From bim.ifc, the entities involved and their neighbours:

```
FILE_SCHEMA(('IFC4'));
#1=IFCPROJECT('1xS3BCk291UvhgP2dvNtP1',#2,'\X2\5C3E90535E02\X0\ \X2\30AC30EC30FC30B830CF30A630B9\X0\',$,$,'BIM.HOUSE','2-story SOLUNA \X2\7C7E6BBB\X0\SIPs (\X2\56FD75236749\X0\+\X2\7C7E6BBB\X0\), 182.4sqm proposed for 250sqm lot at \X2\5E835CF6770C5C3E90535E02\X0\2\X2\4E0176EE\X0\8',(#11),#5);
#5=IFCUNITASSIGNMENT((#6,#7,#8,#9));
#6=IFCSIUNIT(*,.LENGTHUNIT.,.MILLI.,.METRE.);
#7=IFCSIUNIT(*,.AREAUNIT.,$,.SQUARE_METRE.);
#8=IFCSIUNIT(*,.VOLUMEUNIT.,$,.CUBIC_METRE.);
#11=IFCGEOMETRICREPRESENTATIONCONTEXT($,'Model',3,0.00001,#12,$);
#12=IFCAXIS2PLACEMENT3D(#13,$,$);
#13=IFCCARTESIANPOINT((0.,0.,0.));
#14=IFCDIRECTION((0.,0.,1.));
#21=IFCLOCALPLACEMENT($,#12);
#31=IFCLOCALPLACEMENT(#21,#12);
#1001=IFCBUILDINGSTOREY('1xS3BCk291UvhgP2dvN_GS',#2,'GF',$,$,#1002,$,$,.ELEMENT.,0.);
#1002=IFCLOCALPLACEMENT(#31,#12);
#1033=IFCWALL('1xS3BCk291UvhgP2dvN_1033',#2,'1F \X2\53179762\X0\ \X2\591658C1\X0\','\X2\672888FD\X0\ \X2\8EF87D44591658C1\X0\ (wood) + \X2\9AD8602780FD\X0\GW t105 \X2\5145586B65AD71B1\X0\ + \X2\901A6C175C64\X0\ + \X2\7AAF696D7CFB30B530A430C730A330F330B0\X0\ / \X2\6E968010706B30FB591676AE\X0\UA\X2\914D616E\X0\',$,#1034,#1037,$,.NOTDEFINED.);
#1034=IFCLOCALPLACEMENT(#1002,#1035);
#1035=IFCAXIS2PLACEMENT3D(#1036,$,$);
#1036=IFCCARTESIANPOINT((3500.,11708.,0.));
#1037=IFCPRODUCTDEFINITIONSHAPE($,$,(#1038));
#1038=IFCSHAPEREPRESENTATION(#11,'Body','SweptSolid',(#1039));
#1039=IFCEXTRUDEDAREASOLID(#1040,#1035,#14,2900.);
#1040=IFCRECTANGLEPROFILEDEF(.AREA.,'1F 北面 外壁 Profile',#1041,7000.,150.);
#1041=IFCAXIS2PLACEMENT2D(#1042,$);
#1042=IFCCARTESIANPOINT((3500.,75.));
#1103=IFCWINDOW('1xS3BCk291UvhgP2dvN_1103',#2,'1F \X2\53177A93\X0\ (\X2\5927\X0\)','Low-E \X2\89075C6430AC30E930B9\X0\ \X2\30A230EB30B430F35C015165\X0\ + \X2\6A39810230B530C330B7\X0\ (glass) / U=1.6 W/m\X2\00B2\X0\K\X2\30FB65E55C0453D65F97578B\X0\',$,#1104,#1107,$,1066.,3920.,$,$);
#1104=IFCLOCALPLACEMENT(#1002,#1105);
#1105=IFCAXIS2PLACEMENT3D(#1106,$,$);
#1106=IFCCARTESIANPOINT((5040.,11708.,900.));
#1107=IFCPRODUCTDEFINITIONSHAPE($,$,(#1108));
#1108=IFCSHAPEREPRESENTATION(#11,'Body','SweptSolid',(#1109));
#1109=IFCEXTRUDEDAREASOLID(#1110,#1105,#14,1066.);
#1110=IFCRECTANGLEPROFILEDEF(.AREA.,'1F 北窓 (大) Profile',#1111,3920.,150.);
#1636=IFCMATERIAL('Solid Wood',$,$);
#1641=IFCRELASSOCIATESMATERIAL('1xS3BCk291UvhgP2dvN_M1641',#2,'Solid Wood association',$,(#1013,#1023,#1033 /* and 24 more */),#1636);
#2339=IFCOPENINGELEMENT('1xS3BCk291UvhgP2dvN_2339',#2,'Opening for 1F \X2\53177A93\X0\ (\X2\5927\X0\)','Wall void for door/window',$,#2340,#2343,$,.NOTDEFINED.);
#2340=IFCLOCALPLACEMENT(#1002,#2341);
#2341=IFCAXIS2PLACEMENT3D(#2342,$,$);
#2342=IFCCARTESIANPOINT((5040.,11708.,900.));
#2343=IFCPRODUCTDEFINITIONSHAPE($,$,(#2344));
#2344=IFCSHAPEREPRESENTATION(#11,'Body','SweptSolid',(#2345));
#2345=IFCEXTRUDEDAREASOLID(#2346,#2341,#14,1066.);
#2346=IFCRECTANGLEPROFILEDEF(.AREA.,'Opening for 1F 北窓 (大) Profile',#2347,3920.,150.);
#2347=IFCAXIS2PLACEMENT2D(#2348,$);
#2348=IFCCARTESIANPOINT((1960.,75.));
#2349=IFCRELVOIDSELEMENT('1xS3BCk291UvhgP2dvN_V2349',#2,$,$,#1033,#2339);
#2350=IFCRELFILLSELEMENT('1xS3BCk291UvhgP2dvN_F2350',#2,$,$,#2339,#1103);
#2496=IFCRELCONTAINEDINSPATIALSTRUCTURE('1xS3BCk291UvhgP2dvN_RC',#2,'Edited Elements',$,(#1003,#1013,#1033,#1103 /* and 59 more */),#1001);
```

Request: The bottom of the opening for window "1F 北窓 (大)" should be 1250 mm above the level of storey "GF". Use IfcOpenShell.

```python
import numpy as np
import ifcopenshell
import ifcopenshell.api.geometry
import ifcopenshell.geom
import ifcopenshell.util.element
import ifcopenshell.util.placement
import ifcopenshell.util.shape
import ifcopenshell.util.unit

model = ifcopenshell.open("bim.ifc")
unit_scale = ifcopenshell.util.unit.calculate_unit_scale(model)

window = model.by_guid("1xS3BCk291UvhgP2dvN_1103")
opening = window.FillsVoids[0].RelatingOpeningElement
storey = ifcopenshell.util.element.get_container(window, ifc_class="IfcBuildingStorey")
level = ifcopenshell.util.placement.get_local_placement(storey.ObjectPlacement)[2, 3]

# The opening's origin need not be at the sill, so measure its lowest point.
shape = ifcopenshell.geom.create_shape(ifcopenshell.geom.settings(), opening)
bottom = ifcopenshell.util.shape.get_shape_bottom_elevation(shape, shape.geometry) / unit_scale
dz = level + 1.25 / unit_scale - bottom

shift = np.array([0.0, 0.0, dz])
# The window is not placed relative to its opening, so move both.
for product in (opening, window):
    matrix = ifcopenshell.util.placement.get_local_placement(product.ObjectPlacement)
    matrix[:3, 3] += shift
    ifcopenshell.api.geometry.edit_object_placement(model, product=product, matrix=matrix, is_si=False)

print(f"moved by {dz * unit_scale:+.3f} m")

model.write("bim_v2.ifc")
```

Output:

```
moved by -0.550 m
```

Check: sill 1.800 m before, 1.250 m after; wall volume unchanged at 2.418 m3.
